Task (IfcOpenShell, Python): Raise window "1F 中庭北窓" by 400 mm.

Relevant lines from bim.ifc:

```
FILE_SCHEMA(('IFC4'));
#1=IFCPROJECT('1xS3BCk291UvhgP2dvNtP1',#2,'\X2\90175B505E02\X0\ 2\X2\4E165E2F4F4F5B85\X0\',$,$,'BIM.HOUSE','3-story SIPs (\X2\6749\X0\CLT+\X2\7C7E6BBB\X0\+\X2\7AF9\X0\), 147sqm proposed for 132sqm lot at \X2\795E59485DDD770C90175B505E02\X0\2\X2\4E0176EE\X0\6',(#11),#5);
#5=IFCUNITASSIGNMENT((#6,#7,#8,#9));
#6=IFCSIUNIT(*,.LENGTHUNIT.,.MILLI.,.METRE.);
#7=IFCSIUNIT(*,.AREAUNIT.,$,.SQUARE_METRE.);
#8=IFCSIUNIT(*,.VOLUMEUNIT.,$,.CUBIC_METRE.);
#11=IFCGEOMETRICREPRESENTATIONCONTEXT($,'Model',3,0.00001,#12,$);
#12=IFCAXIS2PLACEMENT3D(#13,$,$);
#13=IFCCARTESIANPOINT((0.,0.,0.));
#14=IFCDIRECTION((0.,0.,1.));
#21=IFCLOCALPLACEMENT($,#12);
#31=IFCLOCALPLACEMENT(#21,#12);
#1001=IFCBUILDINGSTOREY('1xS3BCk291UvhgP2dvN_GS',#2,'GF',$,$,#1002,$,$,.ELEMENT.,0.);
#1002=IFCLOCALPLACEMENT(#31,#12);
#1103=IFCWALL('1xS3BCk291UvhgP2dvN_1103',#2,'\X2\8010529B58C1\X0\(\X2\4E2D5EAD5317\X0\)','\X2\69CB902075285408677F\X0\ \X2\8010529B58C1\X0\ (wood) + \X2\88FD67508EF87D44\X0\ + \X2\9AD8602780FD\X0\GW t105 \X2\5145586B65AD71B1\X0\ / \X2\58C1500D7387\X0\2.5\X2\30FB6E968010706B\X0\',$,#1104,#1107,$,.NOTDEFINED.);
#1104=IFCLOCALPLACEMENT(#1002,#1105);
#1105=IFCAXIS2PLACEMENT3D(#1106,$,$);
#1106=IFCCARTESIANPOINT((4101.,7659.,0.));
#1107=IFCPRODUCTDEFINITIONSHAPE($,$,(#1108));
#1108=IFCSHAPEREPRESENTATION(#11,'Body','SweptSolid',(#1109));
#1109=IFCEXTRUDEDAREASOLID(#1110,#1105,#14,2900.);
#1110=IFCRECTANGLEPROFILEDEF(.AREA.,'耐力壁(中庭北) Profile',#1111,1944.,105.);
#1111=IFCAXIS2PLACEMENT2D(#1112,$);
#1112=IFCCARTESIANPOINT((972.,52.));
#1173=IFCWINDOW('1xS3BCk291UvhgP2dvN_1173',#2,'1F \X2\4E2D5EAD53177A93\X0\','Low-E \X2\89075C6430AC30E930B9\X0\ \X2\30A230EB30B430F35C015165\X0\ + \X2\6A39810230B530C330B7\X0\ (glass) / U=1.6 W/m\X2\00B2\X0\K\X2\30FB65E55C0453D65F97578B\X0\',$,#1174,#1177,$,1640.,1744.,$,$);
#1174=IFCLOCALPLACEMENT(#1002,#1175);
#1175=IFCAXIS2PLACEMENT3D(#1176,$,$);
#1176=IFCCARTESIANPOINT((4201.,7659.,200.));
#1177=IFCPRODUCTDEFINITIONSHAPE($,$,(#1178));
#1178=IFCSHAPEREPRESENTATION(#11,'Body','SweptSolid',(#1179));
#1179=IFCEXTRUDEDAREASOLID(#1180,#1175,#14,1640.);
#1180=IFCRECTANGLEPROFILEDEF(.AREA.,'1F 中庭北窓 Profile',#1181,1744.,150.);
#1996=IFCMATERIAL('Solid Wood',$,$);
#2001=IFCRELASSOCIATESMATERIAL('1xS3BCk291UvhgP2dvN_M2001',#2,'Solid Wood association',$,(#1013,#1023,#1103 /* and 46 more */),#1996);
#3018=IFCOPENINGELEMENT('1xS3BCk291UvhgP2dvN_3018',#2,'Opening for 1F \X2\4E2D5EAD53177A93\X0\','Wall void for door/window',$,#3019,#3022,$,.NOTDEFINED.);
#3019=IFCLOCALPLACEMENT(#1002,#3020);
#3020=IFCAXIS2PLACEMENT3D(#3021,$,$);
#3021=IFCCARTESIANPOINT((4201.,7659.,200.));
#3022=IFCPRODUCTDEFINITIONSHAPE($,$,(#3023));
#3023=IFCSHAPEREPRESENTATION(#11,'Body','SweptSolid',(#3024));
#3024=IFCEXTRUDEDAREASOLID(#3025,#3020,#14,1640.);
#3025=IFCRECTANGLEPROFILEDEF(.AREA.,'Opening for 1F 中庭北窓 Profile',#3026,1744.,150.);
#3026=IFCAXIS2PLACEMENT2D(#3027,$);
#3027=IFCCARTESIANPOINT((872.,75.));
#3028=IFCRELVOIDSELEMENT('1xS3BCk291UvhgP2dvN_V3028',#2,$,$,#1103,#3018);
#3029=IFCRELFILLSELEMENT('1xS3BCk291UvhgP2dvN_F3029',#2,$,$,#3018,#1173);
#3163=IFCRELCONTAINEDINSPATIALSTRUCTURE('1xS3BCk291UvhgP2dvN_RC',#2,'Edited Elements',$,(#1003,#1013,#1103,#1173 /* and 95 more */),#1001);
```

```python
import numpy as np
import ifcopenshell
import ifcopenshell.api.geometry
import ifcopenshell.util.placement
import ifcopenshell.util.unit

model = ifcopenshell.open("bim.ifc")
unit_scale = ifcopenshell.util.unit.calculate_unit_scale(model)

window = model.by_id(1173)
opening = window.FillsVoids[0].RelatingOpeningElement
dz = 0.4 / unit_scale

shift = np.array([0.0, 0.0, dz])
# The window is not placed relative to its opening, so move both.
for product in (opening, window):
    matrix = ifcopenshell.util.placement.get_local_placement(product.ObjectPlacement)
    matrix[:3, 3] += shift
    ifcopenshell.api.geometry.edit_object_placement(model, product=product, matrix=matrix, is_si=False)

print(f"moved by {dz * unit_scale:+.3f} m")

model.write("bim_rev.ifc")
```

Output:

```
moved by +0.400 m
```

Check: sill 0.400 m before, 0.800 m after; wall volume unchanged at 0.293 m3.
